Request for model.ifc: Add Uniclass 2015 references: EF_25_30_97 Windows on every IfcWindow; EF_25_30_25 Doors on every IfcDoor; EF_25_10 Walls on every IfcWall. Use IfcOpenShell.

First a look at what the model holds.

```python
import ifcopenshell

model = ifcopenshell.open("model.ifc")
print(model.schema)
print("classifications:", [c.Name for c in model.by_type("IfcClassification")])
for ifc_class in ("IfcDoor", "IfcRoof", "IfcStair", "IfcWall", "IfcWindow"):
    print(ifc_class, len(model.by_type(ifc_class)))
```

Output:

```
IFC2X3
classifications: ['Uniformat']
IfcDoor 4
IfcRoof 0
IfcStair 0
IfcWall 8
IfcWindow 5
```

```python
import ifcopenshell
import ifcopenshell.api.classification

model = ifcopenshell.open("model.ifc")

# IFC2X3 requires Source and Edition and has no link from the project to the system.
system = model.create_entity("IfcClassification", Source="NBS", Edition="2015", Name="Uniclass 2015")

codes = {
    "IfcWindow": ("EF_25_30_97", "Windows"),
    "IfcDoor": ("EF_25_30_25", "Doors"),
    "IfcWall": ("EF_25_10", "Walls"),
}
for ifc_class, (code, name) in codes.items():
    products = model.by_type(ifc_class)
    ifcopenshell.api.classification.add_reference(
        model, products=products, classification=system, identification=code, name=name
    )
    print(code, len(products))

model.write("model_updated.ifc")
```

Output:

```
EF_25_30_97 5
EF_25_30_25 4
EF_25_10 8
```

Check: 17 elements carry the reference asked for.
